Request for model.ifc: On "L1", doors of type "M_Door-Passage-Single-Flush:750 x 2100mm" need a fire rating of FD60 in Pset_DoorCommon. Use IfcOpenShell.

First a look at what the model holds.

```python
import ifcopenshell
import ifcopenshell.util.element

model = ifcopenshell.open("model.ifc")
print(model.schema)
storey = next(s for s in model.by_type("IfcBuildingStorey") if s.Name == "L1")
doors = [e for e in ifcopenshell.util.element.get_decomposition(storey) if e.is_a("IfcDoor")]
seen = {}
for e in doors:
    element_type = ifcopenshell.util.element.get_type(e)
    key = (element_type.Name if element_type != e and element_type else None, ifcopenshell.util.element.get_pset(e, "Pset_DoorCommon", "FireRating"))
    seen[key] = seen.get(key, 0) + 1
for (name, value), count in sorted(seen.items(), key=str):
    print(count, "x", name, "|", value)
```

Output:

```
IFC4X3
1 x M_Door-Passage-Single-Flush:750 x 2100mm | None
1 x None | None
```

```python
import ifcopenshell
import ifcopenshell.api.pset
import ifcopenshell.util.element

model = ifcopenshell.open("model.ifc")

storey = next(s for s in model.by_type("IfcBuildingStorey") if s.Name == "L1")
doors = [e for e in ifcopenshell.util.element.get_decomposition(storey) if e.is_a("IfcDoor")]

count = 0
for e in doors:
    element_type = ifcopenshell.util.element.get_type(e)
    if element_type in (None, e) or element_type.Name != "M_Door-Passage-Single-Flush:750 x 2100mm":
        continue
    # add_pset returns the element's existing set when there is one.
    pset = ifcopenshell.api.pset.add_pset(model, product=e, name="Pset_DoorCommon")
    ifcopenshell.api.pset.edit_pset(model, pset=pset, properties={"FireRating": "FD60"})
    count += 1

print(count, "doors updated")

model.write("model-out.ifc")
```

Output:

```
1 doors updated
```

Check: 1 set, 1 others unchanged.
